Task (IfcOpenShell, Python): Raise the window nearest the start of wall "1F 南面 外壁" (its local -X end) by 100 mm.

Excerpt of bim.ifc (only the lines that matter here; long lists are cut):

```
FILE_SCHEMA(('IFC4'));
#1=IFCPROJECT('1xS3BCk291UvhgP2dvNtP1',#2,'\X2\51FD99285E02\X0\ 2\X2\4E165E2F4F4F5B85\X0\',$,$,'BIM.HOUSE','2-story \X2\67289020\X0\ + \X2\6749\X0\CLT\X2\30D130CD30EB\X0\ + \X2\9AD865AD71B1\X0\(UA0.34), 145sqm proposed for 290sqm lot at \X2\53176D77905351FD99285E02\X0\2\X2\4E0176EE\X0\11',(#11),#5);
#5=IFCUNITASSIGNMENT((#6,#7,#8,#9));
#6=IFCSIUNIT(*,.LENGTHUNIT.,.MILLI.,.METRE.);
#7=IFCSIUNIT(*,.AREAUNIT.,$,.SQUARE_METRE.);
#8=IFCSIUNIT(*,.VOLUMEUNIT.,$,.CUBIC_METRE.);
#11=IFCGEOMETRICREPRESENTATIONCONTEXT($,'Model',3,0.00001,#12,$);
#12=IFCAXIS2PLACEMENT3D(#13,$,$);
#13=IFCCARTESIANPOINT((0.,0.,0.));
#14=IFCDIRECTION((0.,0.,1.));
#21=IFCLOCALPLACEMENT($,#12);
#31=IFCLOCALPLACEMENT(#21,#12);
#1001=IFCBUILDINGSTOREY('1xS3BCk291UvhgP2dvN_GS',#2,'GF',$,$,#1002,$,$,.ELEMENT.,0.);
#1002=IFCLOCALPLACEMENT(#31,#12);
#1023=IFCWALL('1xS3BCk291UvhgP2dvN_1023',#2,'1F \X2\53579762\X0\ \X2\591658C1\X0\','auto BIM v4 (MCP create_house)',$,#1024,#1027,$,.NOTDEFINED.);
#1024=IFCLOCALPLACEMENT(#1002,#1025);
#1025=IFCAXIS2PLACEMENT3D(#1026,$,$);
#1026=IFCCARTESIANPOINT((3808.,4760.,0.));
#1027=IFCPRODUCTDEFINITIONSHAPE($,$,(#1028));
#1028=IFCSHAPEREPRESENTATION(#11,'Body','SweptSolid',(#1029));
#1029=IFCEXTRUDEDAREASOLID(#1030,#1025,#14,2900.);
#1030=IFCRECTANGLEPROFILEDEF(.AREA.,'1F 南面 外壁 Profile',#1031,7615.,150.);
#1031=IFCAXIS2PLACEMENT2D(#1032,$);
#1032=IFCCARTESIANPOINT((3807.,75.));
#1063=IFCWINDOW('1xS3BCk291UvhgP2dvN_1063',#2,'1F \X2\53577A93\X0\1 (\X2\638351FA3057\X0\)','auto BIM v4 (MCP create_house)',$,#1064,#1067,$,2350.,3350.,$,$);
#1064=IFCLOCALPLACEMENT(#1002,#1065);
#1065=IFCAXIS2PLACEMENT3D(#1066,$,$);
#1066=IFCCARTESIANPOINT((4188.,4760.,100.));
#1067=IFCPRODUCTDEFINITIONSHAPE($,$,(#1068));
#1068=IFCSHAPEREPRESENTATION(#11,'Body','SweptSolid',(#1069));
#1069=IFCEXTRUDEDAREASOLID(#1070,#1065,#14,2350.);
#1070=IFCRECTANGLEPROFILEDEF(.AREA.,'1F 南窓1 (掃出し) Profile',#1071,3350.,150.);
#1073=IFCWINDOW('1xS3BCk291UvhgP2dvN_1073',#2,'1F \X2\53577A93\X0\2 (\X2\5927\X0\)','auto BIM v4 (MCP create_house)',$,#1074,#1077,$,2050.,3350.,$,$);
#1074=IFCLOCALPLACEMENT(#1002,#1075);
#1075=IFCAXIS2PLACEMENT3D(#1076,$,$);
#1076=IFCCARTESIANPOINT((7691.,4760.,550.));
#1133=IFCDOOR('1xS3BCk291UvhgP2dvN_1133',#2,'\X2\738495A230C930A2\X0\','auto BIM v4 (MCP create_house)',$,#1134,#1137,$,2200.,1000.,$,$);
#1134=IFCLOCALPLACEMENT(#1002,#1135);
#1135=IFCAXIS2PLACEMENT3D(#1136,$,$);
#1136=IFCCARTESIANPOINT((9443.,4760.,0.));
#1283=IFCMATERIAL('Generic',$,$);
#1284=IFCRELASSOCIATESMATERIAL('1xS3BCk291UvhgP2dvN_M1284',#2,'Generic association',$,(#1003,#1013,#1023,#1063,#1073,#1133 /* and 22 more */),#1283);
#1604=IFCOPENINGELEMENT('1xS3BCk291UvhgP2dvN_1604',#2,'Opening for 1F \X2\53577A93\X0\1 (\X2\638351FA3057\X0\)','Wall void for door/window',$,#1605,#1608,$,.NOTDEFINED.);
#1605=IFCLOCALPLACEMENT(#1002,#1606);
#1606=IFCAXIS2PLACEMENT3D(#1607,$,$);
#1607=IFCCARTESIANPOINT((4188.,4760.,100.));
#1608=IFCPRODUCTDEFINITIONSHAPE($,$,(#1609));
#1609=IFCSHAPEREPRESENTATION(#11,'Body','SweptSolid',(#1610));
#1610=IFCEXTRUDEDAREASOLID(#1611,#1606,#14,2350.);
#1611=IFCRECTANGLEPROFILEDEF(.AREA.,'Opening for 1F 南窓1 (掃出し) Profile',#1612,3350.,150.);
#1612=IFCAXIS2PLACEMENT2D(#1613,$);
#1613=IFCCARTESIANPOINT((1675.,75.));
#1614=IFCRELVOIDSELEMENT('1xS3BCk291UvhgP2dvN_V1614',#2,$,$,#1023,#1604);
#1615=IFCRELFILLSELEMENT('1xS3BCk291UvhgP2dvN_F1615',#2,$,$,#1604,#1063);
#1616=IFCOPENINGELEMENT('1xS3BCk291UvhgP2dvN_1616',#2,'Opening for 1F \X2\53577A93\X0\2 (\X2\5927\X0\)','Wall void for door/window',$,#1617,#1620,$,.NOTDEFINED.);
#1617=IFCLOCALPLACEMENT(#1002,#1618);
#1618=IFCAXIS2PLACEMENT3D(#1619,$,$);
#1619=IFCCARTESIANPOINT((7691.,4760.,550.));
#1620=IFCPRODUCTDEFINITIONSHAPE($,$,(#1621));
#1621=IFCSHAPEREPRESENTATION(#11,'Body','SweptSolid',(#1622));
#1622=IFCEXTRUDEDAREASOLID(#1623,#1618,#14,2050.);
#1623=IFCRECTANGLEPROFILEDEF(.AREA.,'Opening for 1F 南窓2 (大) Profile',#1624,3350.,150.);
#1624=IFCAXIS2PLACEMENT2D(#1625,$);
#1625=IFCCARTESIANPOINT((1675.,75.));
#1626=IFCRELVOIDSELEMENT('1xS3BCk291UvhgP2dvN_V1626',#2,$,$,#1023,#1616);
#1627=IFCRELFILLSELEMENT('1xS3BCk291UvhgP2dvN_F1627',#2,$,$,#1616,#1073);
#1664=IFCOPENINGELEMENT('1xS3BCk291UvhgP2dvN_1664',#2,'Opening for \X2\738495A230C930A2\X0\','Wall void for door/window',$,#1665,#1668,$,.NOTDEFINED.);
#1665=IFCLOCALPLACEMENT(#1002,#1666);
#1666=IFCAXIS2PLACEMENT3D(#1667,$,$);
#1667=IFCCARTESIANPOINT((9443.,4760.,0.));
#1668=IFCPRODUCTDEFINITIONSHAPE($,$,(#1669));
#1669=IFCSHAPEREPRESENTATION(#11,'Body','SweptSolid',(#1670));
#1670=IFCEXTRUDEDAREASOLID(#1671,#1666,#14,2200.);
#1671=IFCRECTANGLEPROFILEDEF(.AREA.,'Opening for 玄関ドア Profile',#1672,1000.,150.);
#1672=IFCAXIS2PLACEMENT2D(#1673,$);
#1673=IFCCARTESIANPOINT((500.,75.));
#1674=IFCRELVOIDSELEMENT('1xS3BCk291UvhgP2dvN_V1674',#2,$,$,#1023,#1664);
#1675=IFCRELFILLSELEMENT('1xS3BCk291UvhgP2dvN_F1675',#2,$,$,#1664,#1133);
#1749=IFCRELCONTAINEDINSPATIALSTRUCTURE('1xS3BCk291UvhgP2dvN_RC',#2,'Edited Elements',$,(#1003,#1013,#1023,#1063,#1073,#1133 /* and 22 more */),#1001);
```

```python
import numpy as np
import ifcopenshell
import ifcopenshell.api.geometry
import ifcopenshell.util.placement
import ifcopenshell.util.unit

model = ifcopenshell.open("bim.ifc")
unit_scale = ifcopenshell.util.unit.calculate_unit_scale(model)

window = model.by_guid("1xS3BCk291UvhgP2dvN_1063")
opening = window.FillsVoids[0].RelatingOpeningElement
dz = 0.1 / unit_scale

shift = np.array([0.0, 0.0, dz])
# The window is not placed relative to its opening, so move both.
for product in (opening, window):
    matrix = ifcopenshell.util.placement.get_local_placement(product.ObjectPlacement)
    matrix[:3, 3] += shift
    ifcopenshell.api.geometry.edit_object_placement(model, product=product, matrix=matrix, is_si=False)

print(f"moved by {dz * unit_scale:+.3f} m")

model.write("bim_updated.ifc")
```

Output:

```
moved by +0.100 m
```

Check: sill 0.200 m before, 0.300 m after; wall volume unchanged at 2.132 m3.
